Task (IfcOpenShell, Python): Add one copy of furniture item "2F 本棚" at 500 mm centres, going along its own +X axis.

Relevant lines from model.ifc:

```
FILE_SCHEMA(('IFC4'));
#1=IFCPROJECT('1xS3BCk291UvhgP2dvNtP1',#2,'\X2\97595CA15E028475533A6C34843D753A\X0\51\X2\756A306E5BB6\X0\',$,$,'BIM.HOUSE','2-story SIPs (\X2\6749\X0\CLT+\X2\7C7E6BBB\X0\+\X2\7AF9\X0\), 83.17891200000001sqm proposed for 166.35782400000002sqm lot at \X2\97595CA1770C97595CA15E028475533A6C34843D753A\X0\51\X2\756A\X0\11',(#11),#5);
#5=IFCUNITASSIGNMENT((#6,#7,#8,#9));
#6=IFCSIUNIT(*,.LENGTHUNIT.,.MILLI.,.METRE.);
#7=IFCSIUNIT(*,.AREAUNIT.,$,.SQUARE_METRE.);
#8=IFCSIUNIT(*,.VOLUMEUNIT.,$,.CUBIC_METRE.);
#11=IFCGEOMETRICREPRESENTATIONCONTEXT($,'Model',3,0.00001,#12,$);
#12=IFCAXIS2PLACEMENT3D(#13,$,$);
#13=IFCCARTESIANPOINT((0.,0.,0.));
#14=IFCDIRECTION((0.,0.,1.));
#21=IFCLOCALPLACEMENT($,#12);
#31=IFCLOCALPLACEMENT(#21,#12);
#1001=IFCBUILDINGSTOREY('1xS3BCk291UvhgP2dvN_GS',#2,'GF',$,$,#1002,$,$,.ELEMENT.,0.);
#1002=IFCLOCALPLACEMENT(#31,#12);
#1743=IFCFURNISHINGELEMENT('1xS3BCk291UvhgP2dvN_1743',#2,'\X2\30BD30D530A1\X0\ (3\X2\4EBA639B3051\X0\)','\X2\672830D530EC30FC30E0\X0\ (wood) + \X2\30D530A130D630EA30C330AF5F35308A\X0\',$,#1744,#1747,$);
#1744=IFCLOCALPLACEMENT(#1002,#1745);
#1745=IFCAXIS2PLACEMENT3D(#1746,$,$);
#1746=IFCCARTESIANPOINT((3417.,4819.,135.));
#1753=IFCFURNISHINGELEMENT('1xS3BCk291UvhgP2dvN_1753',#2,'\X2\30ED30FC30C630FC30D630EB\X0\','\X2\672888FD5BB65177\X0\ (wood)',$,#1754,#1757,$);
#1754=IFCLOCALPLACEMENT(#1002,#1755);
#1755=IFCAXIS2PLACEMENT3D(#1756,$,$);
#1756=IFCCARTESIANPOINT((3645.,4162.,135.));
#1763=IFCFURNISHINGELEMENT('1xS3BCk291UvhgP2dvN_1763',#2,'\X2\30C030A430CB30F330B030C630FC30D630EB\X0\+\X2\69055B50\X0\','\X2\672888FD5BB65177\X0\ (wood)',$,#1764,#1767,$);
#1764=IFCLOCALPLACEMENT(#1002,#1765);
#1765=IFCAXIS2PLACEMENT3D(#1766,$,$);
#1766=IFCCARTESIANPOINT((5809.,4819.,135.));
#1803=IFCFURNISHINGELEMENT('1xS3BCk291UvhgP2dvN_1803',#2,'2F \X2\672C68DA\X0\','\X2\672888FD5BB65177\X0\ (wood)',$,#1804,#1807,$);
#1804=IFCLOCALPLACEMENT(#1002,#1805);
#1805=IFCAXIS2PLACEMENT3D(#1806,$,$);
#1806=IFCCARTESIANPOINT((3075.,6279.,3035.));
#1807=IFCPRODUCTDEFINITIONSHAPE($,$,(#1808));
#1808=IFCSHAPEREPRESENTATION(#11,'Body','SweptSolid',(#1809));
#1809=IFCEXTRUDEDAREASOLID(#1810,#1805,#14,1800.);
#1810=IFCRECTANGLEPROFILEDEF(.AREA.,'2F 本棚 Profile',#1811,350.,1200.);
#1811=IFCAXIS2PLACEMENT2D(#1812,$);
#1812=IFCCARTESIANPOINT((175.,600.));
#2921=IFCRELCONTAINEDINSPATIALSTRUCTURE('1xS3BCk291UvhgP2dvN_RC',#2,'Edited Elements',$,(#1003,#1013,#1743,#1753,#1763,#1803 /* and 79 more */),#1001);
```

```python
import ifcopenshell
import ifcopenshell.api.geometry
import ifcopenshell.api.root
import ifcopenshell.util.element
import ifcopenshell.util.placement
import ifcopenshell.util.unit

model = ifcopenshell.open("model.ifc")
unit_scale = ifcopenshell.util.unit.calculate_unit_scale(model)


def reuse_history(source, copy):
    """copy_class also copies each property set's owner history, people and application; keep the originals."""
    for rel in copy.IsDefinedBy:
        if rel.is_a("IfcRelDefinesByProperties") and (history := rel.RelatingPropertyDefinition.OwnerHistory):
            rel.RelatingPropertyDefinition.OwnerHistory = source.OwnerHistory
            ifcopenshell.util.element.remove_deep2(model, history)


source = model.by_guid("1xS3BCk291UvhgP2dvN_1803")
base = ifcopenshell.util.placement.get_local_placement(source.ObjectPlacement)
step = base[:3, 0] * 0.5 / unit_scale

for i in range(1, 2):
    copy = ifcopenshell.api.root.copy_class(model, product=source)
    copy.Representation = ifcopenshell.util.element.copy_deep(
        model, source.Representation, exclude=["IfcGeometricRepresentationContext", "IfcRepresentationMap"]
    )
    reuse_history(source, copy)
    matrix = base.copy()
    matrix[:3, 3] += i * step
    print("added at", matrix[:3, 3].round(3) + 0.0)
    ifcopenshell.api.geometry.edit_object_placement(model, product=copy, matrix=matrix, is_si=False)

model.write("model_rev.ifc")
```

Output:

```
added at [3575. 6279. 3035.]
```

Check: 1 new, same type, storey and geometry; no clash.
